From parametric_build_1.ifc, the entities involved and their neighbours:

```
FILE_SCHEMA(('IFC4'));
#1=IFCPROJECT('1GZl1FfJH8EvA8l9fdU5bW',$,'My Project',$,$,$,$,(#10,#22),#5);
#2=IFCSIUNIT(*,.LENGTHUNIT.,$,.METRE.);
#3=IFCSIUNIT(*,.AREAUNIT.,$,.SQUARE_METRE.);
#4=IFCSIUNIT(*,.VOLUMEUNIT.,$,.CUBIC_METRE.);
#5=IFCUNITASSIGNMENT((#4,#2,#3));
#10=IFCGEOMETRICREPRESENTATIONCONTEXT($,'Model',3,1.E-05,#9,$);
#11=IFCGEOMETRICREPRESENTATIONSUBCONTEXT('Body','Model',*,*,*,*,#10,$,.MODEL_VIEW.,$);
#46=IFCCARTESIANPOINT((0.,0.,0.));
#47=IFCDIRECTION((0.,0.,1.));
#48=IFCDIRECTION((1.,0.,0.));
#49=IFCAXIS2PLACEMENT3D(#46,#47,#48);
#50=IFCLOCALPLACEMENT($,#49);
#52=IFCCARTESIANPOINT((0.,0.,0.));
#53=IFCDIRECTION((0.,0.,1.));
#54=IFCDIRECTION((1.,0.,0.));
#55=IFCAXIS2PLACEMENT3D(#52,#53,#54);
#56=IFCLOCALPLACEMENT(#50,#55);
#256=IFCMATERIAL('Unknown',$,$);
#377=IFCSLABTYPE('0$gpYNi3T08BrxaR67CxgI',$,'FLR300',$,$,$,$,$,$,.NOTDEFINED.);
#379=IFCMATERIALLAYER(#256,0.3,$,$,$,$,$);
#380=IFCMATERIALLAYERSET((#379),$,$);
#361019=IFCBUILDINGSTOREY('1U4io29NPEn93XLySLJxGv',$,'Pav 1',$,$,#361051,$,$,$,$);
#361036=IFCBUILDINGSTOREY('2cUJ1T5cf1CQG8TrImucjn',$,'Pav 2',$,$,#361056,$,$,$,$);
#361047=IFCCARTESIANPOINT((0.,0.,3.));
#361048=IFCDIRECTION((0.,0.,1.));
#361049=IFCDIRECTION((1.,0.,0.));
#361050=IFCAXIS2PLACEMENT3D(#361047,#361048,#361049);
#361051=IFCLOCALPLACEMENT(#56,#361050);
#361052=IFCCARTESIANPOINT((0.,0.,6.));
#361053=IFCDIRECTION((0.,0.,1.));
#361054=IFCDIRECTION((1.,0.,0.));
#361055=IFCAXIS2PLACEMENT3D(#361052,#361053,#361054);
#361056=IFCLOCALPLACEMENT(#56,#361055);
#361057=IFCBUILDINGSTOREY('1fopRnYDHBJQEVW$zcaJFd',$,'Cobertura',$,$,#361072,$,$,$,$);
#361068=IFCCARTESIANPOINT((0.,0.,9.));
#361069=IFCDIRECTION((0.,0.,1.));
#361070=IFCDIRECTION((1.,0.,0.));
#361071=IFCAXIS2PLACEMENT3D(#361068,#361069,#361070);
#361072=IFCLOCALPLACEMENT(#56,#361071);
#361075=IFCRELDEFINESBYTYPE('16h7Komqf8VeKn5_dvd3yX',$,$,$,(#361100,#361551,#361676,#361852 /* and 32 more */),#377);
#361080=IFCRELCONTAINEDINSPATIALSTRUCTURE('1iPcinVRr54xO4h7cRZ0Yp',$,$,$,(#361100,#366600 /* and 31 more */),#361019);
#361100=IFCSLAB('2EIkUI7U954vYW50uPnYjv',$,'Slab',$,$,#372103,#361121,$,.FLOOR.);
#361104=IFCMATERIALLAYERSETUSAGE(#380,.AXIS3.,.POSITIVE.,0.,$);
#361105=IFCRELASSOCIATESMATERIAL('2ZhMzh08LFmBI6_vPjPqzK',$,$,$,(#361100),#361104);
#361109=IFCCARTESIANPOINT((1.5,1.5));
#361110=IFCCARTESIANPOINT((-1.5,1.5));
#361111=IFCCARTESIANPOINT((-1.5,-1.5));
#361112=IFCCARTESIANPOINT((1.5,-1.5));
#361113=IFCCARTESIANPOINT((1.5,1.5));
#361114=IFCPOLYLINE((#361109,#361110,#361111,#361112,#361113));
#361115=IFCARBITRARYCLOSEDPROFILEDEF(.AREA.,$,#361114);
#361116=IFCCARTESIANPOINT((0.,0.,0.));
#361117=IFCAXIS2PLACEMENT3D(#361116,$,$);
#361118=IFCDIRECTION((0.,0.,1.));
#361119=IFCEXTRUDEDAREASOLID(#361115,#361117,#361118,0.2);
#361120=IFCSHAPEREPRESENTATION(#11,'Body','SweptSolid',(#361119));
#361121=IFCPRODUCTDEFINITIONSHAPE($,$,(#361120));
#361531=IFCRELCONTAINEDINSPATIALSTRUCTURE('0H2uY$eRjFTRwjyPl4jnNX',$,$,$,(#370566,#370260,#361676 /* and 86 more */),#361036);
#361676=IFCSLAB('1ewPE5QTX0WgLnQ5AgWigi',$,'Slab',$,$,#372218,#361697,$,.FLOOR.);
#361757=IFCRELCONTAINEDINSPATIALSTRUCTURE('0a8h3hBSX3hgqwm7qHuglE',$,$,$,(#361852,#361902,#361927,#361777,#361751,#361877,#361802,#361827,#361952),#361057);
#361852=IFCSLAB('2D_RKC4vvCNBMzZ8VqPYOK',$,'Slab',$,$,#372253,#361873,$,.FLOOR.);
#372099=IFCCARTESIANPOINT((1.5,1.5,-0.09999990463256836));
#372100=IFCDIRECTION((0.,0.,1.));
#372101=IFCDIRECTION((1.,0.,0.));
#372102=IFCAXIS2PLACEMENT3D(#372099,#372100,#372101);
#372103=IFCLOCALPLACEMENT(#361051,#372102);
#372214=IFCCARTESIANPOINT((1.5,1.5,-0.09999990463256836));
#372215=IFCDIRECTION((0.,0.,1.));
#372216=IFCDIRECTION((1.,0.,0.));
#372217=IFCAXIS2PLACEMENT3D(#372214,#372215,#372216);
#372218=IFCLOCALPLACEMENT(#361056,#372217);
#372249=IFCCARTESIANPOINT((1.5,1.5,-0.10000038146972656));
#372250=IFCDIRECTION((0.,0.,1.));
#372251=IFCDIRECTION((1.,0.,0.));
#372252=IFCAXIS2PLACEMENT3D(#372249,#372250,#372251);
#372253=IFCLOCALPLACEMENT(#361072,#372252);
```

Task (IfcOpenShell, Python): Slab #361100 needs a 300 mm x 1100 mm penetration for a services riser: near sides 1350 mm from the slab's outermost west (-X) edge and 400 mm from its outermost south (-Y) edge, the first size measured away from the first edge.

```python
import numpy as np
import ifcopenshell
import ifcopenshell.api.feature
import ifcopenshell.api.geometry
import ifcopenshell.api.root
import ifcopenshell.geom
import ifcopenshell.util.placement
import ifcopenshell.util.representation
import ifcopenshell.util.shape
import ifcopenshell.util.unit

model = ifcopenshell.open("parametric_build_1.ifc")
unit_scale = ifcopenshell.util.unit.calculate_unit_scale(model)
settings = ifcopenshell.geom.settings()


def volume(element):
    """Net volume in cubic metres, openings subtracted."""
    shape = ifcopenshell.geom.create_shape(settings, element)
    return ifcopenshell.util.shape.get_volume(shape.geometry)


slab = model.by_guid("2EIkUI7U954vYW50uPnYjv")
before = volume(slab)

# Extent in the slab's own axes, in metres. The edges named are its -X and -Y sides.
slab_shape = ifcopenshell.geom.create_shape(settings, slab)
vertices = ifcopenshell.util.shape.get_vertices(slab_shape.geometry)
x_min, y_min, bottom = vertices.min(axis=0)
top = vertices[:, 2].max()

opening = ifcopenshell.api.root.create_entity(model, ifc_class="IfcOpeningElement", name="Services riser opening", predefined_type="OPENING")
context = ifcopenshell.util.representation.get_context(model, "Model", "Body", "MODEL_VIEW")
width, depth = 0.3, 1.1
outline = [(0.0, 0.0), (width, 0.0), (width, depth), (0.0, depth), (0.0, 0.0)]
# Overshoot both faces by 50 mm so the cut is clean.
shape = ifcopenshell.api.geometry.add_slab_representation(
    model, context=context, depth=top - bottom + 0.1, polyline=outline
)
ifcopenshell.api.geometry.assign_representation(model, product=opening, representation=shape)

matrix = ifcopenshell.util.placement.get_local_placement(slab.ObjectPlacement)
matrix[:, 3] = matrix @ np.append(np.array([x_min + 1.35, y_min + 0.4, bottom - 0.05]) / unit_scale, 1.0)
ifcopenshell.api.geometry.edit_object_placement(model, product=opening, matrix=matrix, is_si=False)
ifcopenshell.api.feature.add_feature(model, feature=opening, element=slab)

after = volume(slab)

print(f"slab volume {before:.3f} -> {after:.3f} m3")

model.write("parametric_build_1_updated.ifc")
```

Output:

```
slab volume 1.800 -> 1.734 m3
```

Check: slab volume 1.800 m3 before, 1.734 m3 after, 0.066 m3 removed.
